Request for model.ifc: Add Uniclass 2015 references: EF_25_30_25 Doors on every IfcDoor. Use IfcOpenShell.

First a look at what the model holds.

```python
import ifcopenshell

model = ifcopenshell.open("model.ifc")
print(model.schema)
print("classifications:", [c.Name for c in model.by_type("IfcClassification")])
for ifc_class in ("IfcDoor", "IfcRoof", "IfcStair", "IfcWall", "IfcWindow"):
    print(ifc_class, len(model.by_type(ifc_class)))
```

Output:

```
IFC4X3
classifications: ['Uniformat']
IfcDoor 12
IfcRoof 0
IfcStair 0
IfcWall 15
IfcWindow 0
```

```python
import ifcopenshell
import ifcopenshell.api.classification

model = ifcopenshell.open("model.ifc")

system = ifcopenshell.api.classification.add_classification(model, classification="Uniclass 2015")

codes = {
    "IfcDoor": ("EF_25_30_25", "Doors"),
}
for ifc_class, (code, name) in codes.items():
    products = model.by_type(ifc_class)
    ifcopenshell.api.classification.add_reference(
        model, products=products, classification=system, identification=code, name=name
    )
    print(code, len(products))

model.write("model-out.ifc")
```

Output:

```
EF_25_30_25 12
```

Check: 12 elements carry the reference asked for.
